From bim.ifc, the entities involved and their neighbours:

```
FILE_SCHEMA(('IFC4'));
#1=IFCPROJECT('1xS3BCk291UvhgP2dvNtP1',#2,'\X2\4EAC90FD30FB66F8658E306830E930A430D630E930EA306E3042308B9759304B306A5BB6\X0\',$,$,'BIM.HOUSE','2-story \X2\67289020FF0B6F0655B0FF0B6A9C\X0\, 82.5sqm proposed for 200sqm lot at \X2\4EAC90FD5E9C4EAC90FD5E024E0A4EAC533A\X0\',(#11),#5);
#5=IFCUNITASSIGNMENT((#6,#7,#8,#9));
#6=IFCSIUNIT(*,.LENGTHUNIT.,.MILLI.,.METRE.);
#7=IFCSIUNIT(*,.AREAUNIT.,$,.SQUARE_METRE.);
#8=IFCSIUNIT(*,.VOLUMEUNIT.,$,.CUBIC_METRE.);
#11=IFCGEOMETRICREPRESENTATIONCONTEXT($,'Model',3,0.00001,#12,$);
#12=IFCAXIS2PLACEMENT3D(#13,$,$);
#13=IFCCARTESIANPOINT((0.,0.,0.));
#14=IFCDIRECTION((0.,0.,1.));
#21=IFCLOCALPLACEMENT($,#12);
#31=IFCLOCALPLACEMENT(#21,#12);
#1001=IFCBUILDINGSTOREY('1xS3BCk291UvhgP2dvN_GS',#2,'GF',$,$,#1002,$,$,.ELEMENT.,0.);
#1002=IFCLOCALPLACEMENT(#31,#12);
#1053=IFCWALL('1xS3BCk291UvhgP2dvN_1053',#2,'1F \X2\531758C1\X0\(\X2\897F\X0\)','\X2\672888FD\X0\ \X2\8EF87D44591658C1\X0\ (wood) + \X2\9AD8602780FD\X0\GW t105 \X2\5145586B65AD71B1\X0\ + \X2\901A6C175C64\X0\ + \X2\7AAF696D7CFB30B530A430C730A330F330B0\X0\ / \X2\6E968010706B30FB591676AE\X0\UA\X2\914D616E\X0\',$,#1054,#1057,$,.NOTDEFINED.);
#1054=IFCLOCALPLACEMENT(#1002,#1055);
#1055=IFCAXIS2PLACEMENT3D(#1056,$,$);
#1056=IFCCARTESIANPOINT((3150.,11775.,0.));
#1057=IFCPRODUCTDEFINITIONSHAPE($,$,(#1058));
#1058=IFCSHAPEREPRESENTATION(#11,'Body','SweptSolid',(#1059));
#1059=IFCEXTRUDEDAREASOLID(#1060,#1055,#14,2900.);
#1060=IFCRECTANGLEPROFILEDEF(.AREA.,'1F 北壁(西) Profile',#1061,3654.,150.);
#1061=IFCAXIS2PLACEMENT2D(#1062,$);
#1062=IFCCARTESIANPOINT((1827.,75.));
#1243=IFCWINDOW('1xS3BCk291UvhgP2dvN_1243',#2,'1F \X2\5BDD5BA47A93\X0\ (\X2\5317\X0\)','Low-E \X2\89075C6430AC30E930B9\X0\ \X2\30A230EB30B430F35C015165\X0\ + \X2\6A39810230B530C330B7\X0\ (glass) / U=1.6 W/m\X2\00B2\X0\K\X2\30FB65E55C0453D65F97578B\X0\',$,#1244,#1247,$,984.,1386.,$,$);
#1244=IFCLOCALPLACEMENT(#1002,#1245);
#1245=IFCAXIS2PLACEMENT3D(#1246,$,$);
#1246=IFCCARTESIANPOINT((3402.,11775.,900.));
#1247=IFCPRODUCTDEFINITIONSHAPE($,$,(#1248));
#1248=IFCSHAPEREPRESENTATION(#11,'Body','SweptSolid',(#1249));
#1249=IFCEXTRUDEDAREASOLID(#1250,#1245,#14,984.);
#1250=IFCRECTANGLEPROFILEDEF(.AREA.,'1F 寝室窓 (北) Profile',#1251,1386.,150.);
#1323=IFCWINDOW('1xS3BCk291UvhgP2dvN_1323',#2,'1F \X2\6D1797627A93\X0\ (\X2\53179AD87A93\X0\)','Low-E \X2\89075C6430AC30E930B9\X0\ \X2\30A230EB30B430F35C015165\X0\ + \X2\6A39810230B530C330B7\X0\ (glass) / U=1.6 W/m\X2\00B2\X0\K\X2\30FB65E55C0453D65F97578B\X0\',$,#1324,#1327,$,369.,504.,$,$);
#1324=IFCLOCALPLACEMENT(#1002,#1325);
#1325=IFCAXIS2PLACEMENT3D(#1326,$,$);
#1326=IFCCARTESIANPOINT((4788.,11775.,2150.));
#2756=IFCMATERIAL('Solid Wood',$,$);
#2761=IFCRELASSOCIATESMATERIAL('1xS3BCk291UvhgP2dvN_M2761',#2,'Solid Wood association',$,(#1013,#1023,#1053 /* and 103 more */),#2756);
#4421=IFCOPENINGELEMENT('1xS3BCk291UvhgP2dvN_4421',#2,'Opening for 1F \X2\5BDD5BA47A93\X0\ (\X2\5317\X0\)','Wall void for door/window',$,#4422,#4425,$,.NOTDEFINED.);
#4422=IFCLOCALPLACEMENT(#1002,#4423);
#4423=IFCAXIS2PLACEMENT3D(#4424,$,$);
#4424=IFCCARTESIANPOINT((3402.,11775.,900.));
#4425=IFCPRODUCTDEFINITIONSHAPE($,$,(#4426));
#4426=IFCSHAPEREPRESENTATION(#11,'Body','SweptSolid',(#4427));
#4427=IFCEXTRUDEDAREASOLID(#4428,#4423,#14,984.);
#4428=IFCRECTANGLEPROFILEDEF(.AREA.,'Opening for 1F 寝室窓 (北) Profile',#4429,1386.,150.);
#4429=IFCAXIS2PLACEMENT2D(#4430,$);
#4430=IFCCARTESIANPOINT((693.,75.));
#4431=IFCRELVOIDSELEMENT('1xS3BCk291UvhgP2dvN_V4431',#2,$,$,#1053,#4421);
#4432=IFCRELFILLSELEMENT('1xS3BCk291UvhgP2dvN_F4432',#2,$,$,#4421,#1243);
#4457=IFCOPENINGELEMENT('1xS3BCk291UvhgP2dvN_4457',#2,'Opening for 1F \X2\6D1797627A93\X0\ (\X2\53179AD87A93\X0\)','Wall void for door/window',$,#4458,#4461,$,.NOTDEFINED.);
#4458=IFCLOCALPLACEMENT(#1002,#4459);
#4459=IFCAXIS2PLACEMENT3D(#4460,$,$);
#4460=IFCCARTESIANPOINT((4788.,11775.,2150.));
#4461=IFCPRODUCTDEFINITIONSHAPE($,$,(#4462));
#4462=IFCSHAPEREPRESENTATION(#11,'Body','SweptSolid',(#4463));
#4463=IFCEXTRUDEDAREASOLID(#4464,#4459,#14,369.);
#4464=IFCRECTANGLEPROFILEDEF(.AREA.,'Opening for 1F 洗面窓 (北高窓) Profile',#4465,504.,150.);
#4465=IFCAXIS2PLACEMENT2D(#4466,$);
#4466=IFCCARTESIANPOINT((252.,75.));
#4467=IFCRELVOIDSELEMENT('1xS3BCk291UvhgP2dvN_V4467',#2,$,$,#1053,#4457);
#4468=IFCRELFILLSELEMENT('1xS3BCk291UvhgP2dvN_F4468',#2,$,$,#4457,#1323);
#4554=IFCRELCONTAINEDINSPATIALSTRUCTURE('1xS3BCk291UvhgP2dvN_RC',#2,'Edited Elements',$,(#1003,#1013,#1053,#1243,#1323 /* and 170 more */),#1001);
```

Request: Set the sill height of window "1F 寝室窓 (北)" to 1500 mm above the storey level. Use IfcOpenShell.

```python
import numpy as np
import ifcopenshell
import ifcopenshell.api.geometry
import ifcopenshell.geom
import ifcopenshell.util.element
import ifcopenshell.util.placement
import ifcopenshell.util.shape
import ifcopenshell.util.unit

model = ifcopenshell.open("bim.ifc")
unit_scale = ifcopenshell.util.unit.calculate_unit_scale(model)

window = model.by_guid("1xS3BCk291UvhgP2dvN_1243")
opening = window.FillsVoids[0].RelatingOpeningElement
storey = ifcopenshell.util.element.get_container(window, ifc_class="IfcBuildingStorey")
level = ifcopenshell.util.placement.get_local_placement(storey.ObjectPlacement)[2, 3]

# The opening's origin need not be at the sill, so measure its lowest point.
shape = ifcopenshell.geom.create_shape(ifcopenshell.geom.settings(), opening)
bottom = ifcopenshell.util.shape.get_shape_bottom_elevation(shape, shape.geometry) / unit_scale
dz = level + 1500.0 - bottom

shift = np.array([0.0, 0.0, dz])
# The window is not placed relative to its opening, so move both.
for product in (opening, window):
    matrix = ifcopenshell.util.placement.get_local_placement(product.ObjectPlacement)
    matrix[:3, 3] += shift
    ifcopenshell.api.geometry.edit_object_placement(model, product=product, matrix=matrix, is_si=False)

print(f"moved by {dz * unit_scale:+.3f} m")

model.write("bim_v2.ifc")
```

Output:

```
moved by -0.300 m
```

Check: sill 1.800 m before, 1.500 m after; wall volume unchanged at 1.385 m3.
